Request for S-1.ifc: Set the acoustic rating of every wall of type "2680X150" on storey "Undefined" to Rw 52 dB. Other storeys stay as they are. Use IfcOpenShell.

First a look at what the model holds.

```python
import ifcopenshell
import ifcopenshell.util.element

model = ifcopenshell.open("S-1.ifc")
print(model.schema)
storey = next(s for s in model.by_type("IfcBuildingStorey") if s.Name == "Undefined")
walls = [e for e in ifcopenshell.util.element.get_decomposition(storey) if e.is_a("IfcWall")]
seen = {}
for e in walls:
    element_type = ifcopenshell.util.element.get_type(e)
    key = (element_type.Name if element_type != e and element_type else None, ifcopenshell.util.element.get_pset(e, "Pset_WallCommon", "AcousticRating"))
    seen[key] = seen.get(key, 0) + 1
for (name, value), count in sorted(seen.items(), key=str):
    print(count, "x", name, "|", value)
```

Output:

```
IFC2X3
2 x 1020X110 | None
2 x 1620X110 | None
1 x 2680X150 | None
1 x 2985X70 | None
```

```python
import ifcopenshell
import ifcopenshell.api.pset
import ifcopenshell.util.element

model = ifcopenshell.open("S-1.ifc")

storey = next(s for s in model.by_type("IfcBuildingStorey") if s.Name == "Undefined")
walls = [e for e in ifcopenshell.util.element.get_decomposition(storey) if e.is_a("IfcWall")]

count = 0
for e in walls:
    element_type = ifcopenshell.util.element.get_type(e)
    if element_type in (None, e) or element_type.Name != "2680X150":
        continue
    # add_pset returns the element's existing set when there is one.
    pset = ifcopenshell.api.pset.add_pset(model, product=e, name="Pset_WallCommon")
    ifcopenshell.api.pset.edit_pset(model, pset=pset, properties={"AcousticRating": "Rw 52 dB"})
    count += 1

print(count, "walls updated")

model.write("S-1-out.ifc")
```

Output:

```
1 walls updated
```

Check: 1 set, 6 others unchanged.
